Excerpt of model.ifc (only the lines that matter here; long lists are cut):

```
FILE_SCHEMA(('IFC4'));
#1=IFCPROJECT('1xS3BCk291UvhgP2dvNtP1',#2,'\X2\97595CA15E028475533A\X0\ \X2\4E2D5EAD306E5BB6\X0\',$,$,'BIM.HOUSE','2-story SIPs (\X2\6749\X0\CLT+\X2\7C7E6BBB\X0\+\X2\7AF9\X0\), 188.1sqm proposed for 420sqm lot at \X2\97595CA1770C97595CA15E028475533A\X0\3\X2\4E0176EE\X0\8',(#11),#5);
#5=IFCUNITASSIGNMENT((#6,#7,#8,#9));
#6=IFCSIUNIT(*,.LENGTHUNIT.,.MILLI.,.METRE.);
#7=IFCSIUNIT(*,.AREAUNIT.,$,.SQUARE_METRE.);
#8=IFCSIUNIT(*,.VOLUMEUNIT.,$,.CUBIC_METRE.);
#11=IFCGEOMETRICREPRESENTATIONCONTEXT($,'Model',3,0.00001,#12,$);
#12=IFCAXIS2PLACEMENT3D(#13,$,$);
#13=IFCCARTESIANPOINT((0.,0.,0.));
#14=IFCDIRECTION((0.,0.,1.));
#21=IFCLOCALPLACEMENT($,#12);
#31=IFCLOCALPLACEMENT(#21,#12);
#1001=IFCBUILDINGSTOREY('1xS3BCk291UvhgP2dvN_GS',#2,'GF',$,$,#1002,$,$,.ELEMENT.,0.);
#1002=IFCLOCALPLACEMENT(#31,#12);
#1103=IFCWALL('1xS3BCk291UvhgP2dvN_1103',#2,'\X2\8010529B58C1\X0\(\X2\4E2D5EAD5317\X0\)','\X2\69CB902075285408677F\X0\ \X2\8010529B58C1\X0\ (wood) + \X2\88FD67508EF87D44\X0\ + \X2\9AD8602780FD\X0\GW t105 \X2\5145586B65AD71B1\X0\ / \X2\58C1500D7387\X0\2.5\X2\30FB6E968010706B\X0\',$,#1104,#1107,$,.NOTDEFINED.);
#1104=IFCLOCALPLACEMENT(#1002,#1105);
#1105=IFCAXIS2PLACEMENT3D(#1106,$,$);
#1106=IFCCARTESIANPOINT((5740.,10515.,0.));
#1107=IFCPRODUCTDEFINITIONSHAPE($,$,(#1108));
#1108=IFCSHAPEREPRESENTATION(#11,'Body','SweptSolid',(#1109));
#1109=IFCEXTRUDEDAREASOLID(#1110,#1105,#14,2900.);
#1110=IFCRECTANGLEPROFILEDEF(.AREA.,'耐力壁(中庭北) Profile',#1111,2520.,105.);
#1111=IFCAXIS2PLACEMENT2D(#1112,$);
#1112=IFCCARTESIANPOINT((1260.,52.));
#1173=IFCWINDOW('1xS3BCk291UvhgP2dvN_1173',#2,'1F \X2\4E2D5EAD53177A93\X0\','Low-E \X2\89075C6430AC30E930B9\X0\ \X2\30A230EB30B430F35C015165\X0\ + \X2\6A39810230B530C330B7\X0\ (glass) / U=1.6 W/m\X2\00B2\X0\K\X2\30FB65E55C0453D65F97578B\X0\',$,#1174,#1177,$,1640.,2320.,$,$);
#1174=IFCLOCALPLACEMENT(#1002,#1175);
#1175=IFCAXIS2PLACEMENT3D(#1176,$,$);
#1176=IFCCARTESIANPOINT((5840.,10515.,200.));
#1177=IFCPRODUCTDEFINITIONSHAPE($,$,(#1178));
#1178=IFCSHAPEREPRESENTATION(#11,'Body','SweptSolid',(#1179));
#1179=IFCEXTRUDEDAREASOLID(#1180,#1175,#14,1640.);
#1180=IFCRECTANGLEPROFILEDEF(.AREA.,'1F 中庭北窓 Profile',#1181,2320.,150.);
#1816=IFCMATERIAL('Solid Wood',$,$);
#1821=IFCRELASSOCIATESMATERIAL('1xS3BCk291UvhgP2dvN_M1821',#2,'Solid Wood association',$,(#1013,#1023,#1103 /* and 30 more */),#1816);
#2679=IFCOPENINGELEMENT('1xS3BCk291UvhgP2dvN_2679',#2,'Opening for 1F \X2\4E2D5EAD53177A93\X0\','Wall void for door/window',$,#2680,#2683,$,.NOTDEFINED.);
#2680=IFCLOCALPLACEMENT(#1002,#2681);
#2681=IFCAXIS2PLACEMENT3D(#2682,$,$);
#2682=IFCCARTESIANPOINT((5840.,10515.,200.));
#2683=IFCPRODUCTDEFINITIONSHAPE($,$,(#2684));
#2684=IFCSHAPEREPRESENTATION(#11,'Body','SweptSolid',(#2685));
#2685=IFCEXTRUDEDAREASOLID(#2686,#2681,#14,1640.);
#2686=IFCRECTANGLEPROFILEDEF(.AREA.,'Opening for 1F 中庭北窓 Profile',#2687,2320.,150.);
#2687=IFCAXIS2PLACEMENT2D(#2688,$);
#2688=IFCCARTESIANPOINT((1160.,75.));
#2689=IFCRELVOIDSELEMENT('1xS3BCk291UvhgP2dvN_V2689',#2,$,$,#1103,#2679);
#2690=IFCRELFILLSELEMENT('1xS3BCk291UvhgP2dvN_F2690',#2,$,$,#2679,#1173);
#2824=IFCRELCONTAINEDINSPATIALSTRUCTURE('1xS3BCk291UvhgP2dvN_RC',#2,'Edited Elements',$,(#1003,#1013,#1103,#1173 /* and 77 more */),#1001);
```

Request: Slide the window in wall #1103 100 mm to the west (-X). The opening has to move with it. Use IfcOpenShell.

```python
import ifcopenshell
import ifcopenshell.api.geometry
import ifcopenshell.util.placement
import ifcopenshell.util.unit

model = ifcopenshell.open("model.ifc")
unit_scale = ifcopenshell.util.unit.calculate_unit_scale(model)

window = model.by_guid("1xS3BCk291UvhgP2dvN_1173")
opening = window.FillsVoids[0].RelatingOpeningElement
wall = opening.VoidsElements[0].RelatingBuildingElement

wall_matrix = ifcopenshell.util.placement.get_local_placement(wall.ObjectPlacement)
shift = wall_matrix[:3, 0] * -0.1 / unit_scale
before = ifcopenshell.util.placement.get_local_placement(window.ObjectPlacement)[:3, 3].copy()

# The window is not placed relative to its opening, so move both.
for product in (opening, window):
    matrix = ifcopenshell.util.placement.get_local_placement(product.ObjectPlacement)
    matrix[:3, 3] += shift
    ifcopenshell.api.geometry.edit_object_placement(model, product=product, matrix=matrix, is_si=False)

after = ifcopenshell.util.placement.get_local_placement(window.ObjectPlacement)[:3, 3]
print("window moved by", (after - before).round(3) + 0.0)

model.write("model-out.ifc")
```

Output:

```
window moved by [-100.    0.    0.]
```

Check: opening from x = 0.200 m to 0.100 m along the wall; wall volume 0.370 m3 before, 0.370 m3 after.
